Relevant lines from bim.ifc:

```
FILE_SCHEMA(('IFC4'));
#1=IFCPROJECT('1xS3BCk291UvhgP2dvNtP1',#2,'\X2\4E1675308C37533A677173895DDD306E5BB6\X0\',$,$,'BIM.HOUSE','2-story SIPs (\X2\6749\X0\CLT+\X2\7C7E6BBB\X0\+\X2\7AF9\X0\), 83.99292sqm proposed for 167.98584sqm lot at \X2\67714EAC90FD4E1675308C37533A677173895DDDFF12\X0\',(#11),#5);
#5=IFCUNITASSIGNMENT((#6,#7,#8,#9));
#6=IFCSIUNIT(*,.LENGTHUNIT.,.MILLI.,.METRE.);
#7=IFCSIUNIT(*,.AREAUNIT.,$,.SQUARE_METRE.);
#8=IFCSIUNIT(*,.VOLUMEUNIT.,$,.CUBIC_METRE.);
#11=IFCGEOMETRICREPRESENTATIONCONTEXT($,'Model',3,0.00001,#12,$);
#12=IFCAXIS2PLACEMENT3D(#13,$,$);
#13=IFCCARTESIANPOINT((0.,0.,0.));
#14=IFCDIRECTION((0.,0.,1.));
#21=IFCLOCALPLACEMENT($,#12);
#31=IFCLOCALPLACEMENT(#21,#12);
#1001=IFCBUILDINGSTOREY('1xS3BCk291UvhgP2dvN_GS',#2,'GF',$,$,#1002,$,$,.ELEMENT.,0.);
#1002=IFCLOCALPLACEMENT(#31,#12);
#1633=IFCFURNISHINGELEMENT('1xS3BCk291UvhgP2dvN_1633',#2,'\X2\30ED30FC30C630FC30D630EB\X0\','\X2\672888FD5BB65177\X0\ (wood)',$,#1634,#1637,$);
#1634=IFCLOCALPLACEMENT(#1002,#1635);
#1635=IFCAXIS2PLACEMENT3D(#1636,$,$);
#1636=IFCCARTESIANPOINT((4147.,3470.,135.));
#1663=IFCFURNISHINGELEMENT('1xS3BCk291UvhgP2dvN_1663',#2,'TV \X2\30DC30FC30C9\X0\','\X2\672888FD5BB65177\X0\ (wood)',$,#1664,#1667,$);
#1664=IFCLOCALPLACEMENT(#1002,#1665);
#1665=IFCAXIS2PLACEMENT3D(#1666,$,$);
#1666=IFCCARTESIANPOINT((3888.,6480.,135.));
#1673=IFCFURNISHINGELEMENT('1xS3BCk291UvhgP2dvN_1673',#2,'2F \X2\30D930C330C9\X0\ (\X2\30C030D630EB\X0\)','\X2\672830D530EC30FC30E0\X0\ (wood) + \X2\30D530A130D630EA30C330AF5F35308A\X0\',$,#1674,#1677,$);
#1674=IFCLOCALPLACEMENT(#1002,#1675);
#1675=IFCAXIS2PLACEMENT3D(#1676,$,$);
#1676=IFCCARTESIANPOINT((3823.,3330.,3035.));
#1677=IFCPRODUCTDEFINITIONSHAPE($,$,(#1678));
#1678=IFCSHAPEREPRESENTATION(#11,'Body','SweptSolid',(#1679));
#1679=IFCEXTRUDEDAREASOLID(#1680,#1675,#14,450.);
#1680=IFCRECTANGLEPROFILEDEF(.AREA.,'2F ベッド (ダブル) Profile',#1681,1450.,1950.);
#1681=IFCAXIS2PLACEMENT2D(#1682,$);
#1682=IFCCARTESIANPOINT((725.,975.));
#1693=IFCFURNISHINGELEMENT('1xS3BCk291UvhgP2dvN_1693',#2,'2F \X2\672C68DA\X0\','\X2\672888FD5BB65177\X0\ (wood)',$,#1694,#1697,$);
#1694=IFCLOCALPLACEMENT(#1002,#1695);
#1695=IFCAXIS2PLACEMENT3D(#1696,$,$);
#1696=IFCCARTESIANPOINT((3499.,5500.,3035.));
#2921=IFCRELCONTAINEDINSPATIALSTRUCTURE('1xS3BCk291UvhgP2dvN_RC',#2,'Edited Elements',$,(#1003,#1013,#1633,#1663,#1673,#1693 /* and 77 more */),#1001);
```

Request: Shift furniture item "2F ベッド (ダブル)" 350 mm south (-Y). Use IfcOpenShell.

```python
import ifcopenshell
import ifcopenshell.api.geometry
import ifcopenshell.util.placement

model = ifcopenshell.open("bim.ifc")

item = model.by_guid("1xS3BCk291UvhgP2dvN_1673")
matrix = ifcopenshell.util.placement.get_local_placement(item.ObjectPlacement)
matrix[1, 3] -= 350.0
ifcopenshell.api.geometry.edit_object_placement(model, product=item, matrix=matrix, is_si=False)

print(ifcopenshell.util.placement.get_local_placement(item.ObjectPlacement).round(3) + 0.0)

model.write("bim_v2.ifc")
```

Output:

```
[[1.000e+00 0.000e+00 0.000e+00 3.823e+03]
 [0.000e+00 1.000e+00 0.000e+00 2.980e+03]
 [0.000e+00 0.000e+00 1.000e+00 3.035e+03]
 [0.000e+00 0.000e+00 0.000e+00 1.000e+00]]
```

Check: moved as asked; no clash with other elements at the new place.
